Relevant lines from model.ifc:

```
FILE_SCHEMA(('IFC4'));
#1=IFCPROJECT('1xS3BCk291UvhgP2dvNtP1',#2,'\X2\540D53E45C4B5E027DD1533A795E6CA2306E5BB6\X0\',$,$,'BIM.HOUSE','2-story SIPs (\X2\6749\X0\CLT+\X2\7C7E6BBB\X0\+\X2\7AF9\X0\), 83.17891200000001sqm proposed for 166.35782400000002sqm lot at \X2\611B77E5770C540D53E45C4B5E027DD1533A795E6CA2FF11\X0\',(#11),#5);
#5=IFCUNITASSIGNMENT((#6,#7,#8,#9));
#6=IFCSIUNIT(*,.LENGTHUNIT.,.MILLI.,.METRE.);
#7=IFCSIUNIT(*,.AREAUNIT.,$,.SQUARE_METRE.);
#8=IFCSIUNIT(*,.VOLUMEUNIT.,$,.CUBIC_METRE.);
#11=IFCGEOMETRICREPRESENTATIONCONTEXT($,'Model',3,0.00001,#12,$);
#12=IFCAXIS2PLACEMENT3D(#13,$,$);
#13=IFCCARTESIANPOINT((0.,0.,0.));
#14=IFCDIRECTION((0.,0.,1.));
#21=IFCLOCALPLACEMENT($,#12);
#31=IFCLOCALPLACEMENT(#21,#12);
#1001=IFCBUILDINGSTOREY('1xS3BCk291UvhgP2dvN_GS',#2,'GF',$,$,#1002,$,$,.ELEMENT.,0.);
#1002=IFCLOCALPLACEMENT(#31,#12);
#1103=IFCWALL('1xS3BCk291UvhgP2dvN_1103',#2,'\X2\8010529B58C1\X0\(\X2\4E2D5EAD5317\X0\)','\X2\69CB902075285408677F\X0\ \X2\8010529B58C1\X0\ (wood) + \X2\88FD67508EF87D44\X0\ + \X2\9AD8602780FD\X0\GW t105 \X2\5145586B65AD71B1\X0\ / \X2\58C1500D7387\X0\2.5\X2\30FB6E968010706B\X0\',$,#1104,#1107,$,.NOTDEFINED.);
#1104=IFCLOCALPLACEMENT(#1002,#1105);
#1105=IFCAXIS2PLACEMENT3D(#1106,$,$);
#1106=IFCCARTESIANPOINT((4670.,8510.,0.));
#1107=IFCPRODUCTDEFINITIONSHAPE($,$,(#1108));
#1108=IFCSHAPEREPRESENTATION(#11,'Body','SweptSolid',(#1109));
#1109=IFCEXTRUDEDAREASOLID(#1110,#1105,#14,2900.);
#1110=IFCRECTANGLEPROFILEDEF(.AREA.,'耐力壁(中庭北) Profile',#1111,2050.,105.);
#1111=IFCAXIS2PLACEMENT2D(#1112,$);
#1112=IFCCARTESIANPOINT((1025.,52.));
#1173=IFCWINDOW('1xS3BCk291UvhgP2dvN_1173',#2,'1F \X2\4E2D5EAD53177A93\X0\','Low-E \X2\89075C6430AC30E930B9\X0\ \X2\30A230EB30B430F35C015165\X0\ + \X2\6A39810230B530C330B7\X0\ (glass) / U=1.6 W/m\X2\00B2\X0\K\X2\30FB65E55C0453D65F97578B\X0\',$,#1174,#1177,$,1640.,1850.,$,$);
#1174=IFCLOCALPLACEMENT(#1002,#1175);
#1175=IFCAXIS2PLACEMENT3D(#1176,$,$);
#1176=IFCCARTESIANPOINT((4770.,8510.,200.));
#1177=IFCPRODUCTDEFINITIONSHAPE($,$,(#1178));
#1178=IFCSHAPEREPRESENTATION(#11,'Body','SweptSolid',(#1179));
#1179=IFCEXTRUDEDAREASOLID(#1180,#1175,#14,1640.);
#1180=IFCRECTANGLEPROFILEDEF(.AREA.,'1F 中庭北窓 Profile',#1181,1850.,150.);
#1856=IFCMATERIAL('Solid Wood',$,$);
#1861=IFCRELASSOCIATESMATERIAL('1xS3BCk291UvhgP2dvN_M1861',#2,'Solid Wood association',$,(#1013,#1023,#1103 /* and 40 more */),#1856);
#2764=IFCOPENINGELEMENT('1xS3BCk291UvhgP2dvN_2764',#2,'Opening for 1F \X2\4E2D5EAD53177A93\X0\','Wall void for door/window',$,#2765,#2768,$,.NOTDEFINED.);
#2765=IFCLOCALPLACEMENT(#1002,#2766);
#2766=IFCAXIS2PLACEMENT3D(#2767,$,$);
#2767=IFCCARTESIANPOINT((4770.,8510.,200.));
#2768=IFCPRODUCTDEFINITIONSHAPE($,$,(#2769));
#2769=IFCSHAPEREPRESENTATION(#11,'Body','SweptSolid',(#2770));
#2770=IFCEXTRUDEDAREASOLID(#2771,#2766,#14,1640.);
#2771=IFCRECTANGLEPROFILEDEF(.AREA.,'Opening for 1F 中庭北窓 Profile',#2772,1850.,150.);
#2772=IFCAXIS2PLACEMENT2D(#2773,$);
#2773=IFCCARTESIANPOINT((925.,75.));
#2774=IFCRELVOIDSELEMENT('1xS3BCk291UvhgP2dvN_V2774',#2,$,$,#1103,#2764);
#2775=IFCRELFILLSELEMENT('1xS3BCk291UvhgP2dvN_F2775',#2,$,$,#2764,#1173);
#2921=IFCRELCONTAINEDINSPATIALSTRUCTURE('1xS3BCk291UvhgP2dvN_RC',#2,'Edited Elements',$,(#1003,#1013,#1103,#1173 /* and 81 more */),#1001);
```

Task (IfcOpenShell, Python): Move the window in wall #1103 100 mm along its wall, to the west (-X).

```python
import ifcopenshell
import ifcopenshell.api.geometry
import ifcopenshell.util.placement

model = ifcopenshell.open("model.ifc")

window = model.by_guid("1xS3BCk291UvhgP2dvN_1173")
opening = window.FillsVoids[0].RelatingOpeningElement
wall = opening.VoidsElements[0].RelatingBuildingElement

wall_matrix = ifcopenshell.util.placement.get_local_placement(wall.ObjectPlacement)
shift = wall_matrix[:3, 0] * -100.0
before = ifcopenshell.util.placement.get_local_placement(window.ObjectPlacement)[:3, 3].copy()

# The window is not placed relative to its opening, so move both.
for product in (opening, window):
    matrix = ifcopenshell.util.placement.get_local_placement(product.ObjectPlacement)
    matrix[:3, 3] += shift
    ifcopenshell.api.geometry.edit_object_placement(model, product=product, matrix=matrix, is_si=False)

after = ifcopenshell.util.placement.get_local_placement(window.ObjectPlacement)[:3, 3]
print("window moved by", (after - before).round(3) + 0.0)

model.write("model_rev.ifc")
```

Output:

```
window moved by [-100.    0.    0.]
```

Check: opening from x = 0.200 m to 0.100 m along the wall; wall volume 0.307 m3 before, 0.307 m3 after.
